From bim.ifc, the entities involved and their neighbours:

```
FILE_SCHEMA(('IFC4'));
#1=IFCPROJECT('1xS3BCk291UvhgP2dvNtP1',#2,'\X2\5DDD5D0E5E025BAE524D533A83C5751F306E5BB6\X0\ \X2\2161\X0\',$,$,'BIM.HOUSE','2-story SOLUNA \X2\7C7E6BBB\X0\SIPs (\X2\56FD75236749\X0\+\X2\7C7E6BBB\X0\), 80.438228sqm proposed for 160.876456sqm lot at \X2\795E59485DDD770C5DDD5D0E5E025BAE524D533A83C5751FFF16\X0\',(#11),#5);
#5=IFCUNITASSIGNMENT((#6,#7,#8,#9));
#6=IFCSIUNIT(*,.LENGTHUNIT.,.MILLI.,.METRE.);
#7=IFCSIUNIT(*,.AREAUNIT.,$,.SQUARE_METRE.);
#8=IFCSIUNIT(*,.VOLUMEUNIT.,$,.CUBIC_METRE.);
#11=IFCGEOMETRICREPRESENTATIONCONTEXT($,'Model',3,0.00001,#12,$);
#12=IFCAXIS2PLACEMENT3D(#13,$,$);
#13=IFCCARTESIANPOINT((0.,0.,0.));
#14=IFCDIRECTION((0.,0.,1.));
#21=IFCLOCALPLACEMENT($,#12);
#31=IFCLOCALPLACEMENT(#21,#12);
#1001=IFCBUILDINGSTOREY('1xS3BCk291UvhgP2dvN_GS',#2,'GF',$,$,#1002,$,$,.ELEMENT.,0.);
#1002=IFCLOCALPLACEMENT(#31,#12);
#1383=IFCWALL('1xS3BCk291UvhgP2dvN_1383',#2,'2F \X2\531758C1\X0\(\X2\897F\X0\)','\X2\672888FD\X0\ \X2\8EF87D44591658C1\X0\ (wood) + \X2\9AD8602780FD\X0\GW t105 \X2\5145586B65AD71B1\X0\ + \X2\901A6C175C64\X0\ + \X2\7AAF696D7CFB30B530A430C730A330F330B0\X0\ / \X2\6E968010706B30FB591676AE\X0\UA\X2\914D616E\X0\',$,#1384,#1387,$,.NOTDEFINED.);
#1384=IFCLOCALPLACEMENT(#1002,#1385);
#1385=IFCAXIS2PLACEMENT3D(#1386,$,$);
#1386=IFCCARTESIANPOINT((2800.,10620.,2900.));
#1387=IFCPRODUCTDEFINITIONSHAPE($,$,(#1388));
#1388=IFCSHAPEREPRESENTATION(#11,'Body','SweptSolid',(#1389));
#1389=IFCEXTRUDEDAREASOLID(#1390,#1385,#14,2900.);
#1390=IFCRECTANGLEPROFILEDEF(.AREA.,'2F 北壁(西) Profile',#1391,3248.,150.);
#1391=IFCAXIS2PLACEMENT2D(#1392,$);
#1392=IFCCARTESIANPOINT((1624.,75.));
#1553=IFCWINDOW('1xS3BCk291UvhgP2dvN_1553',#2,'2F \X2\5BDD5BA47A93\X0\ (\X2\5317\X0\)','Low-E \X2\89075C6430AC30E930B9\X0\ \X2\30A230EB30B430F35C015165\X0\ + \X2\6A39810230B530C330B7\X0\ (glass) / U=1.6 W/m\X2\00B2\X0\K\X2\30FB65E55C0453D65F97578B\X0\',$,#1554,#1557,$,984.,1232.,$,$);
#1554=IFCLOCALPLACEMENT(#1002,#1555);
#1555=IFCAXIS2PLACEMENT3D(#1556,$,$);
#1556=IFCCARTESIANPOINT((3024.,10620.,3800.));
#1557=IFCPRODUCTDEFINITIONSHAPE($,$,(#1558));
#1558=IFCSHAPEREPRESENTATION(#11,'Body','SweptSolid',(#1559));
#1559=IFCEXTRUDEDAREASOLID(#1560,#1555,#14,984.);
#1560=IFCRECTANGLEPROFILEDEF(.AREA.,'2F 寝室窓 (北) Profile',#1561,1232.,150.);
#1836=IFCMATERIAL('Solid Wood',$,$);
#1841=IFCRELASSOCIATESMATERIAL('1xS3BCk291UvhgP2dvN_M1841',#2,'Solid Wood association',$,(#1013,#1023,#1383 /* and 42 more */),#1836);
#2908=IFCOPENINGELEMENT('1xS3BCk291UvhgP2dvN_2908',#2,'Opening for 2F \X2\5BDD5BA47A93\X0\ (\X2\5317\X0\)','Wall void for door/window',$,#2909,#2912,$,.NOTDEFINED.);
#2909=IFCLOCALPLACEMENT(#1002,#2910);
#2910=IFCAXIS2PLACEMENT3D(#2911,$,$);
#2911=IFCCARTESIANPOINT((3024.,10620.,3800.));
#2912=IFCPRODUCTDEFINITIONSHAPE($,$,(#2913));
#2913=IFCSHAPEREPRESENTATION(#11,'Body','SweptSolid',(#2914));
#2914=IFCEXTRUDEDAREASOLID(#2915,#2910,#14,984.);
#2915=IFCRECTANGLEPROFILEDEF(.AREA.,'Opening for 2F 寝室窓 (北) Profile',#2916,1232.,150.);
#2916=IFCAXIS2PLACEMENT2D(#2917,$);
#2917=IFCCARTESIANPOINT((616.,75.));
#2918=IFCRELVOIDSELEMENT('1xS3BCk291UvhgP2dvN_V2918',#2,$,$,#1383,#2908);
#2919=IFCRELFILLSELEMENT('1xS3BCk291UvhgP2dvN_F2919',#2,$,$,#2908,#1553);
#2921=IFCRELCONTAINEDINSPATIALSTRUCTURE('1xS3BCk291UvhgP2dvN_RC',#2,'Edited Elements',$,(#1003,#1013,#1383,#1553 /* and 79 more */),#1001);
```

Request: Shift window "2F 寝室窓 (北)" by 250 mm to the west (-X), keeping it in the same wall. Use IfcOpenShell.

```python
import ifcopenshell
import ifcopenshell.api.geometry
import ifcopenshell.util.placement
import ifcopenshell.util.unit

model = ifcopenshell.open("bim.ifc")
unit_scale = ifcopenshell.util.unit.calculate_unit_scale(model)

window = model.by_guid("1xS3BCk291UvhgP2dvN_1553")
opening = window.FillsVoids[0].RelatingOpeningElement
wall = opening.VoidsElements[0].RelatingBuildingElement

wall_matrix = ifcopenshell.util.placement.get_local_placement(wall.ObjectPlacement)
shift = wall_matrix[:3, 0] * -0.25 / unit_scale
before = ifcopenshell.util.placement.get_local_placement(window.ObjectPlacement)[:3, 3].copy()

# The window is not placed relative to its opening, so move both.
for product in (opening, window):
    matrix = ifcopenshell.util.placement.get_local_placement(product.ObjectPlacement)
    matrix[:3, 3] += shift
    ifcopenshell.api.geometry.edit_object_placement(model, product=product, matrix=matrix, is_si=False)

after = ifcopenshell.util.placement.get_local_placement(window.ObjectPlacement)[:3, 3]
print("window moved by", (after - before).round(3) + 0.0)

model.write("bim-out.ifc")
```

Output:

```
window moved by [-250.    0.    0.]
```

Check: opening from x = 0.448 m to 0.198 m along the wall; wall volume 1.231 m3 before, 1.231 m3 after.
